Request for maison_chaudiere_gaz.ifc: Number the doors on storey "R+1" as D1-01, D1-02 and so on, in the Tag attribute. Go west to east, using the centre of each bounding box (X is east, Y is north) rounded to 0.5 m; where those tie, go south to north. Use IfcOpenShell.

First a look at what the model holds.

```python
import ifcopenshell
import ifcopenshell.util.element
import ifcopenshell.util.placement

model = ifcopenshell.open("maison_chaudiere_gaz.ifc")
print(model.schema)
storey = next(s for s in model.by_type("IfcBuildingStorey") if s.Name == "R+1")
doors = [e for e in ifcopenshell.util.element.get_decomposition(storey) if e.is_a("IfcDoor")]
for e in sorted(doors, key=lambda e: e.id()):
    origin = ifcopenshell.util.placement.get_local_placement(e.ObjectPlacement)[:3, 3]
    print(e.id(), e.Tag, e.Name, origin.round(2) + 0.0, sep=" | ")
```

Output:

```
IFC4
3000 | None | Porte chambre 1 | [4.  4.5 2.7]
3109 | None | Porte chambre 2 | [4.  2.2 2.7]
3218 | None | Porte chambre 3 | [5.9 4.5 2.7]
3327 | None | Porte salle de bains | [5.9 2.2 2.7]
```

```python
import ifcopenshell
import ifcopenshell.geom
import ifcopenshell.util.element
import ifcopenshell.util.shape

model = ifcopenshell.open("maison_chaudiere_gaz.ifc")
settings = ifcopenshell.geom.settings()
settings.set("use-world-coords", True)


def centre(element):
    shape = ifcopenshell.geom.create_shape(settings, element)
    return ifcopenshell.util.shape.get_bbox_centroid(shape.geometry)


storey = next(s for s in model.by_type("IfcBuildingStorey") if s.Name == "R+1")
doors = [e for e in ifcopenshell.util.element.get_decomposition(storey) if e.is_a("IfcDoor")]

# Insertion points can sit at a corner or the storey origin, so sort by the geometry (in metres).
centres = {e: centre(e) for e in doors}
doors.sort(key=lambda e: (round(centres[e][0] / 0.5), centres[e][1]))

for i, e in enumerate(doors, start=1):
    number = f"D1-{i:02d}"
    e.Tag = number
    print(e.id(), number)

model.write("maison_chaudiere_gaz-out.ifc")
```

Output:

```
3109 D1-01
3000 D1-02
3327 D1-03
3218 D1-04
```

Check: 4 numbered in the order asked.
